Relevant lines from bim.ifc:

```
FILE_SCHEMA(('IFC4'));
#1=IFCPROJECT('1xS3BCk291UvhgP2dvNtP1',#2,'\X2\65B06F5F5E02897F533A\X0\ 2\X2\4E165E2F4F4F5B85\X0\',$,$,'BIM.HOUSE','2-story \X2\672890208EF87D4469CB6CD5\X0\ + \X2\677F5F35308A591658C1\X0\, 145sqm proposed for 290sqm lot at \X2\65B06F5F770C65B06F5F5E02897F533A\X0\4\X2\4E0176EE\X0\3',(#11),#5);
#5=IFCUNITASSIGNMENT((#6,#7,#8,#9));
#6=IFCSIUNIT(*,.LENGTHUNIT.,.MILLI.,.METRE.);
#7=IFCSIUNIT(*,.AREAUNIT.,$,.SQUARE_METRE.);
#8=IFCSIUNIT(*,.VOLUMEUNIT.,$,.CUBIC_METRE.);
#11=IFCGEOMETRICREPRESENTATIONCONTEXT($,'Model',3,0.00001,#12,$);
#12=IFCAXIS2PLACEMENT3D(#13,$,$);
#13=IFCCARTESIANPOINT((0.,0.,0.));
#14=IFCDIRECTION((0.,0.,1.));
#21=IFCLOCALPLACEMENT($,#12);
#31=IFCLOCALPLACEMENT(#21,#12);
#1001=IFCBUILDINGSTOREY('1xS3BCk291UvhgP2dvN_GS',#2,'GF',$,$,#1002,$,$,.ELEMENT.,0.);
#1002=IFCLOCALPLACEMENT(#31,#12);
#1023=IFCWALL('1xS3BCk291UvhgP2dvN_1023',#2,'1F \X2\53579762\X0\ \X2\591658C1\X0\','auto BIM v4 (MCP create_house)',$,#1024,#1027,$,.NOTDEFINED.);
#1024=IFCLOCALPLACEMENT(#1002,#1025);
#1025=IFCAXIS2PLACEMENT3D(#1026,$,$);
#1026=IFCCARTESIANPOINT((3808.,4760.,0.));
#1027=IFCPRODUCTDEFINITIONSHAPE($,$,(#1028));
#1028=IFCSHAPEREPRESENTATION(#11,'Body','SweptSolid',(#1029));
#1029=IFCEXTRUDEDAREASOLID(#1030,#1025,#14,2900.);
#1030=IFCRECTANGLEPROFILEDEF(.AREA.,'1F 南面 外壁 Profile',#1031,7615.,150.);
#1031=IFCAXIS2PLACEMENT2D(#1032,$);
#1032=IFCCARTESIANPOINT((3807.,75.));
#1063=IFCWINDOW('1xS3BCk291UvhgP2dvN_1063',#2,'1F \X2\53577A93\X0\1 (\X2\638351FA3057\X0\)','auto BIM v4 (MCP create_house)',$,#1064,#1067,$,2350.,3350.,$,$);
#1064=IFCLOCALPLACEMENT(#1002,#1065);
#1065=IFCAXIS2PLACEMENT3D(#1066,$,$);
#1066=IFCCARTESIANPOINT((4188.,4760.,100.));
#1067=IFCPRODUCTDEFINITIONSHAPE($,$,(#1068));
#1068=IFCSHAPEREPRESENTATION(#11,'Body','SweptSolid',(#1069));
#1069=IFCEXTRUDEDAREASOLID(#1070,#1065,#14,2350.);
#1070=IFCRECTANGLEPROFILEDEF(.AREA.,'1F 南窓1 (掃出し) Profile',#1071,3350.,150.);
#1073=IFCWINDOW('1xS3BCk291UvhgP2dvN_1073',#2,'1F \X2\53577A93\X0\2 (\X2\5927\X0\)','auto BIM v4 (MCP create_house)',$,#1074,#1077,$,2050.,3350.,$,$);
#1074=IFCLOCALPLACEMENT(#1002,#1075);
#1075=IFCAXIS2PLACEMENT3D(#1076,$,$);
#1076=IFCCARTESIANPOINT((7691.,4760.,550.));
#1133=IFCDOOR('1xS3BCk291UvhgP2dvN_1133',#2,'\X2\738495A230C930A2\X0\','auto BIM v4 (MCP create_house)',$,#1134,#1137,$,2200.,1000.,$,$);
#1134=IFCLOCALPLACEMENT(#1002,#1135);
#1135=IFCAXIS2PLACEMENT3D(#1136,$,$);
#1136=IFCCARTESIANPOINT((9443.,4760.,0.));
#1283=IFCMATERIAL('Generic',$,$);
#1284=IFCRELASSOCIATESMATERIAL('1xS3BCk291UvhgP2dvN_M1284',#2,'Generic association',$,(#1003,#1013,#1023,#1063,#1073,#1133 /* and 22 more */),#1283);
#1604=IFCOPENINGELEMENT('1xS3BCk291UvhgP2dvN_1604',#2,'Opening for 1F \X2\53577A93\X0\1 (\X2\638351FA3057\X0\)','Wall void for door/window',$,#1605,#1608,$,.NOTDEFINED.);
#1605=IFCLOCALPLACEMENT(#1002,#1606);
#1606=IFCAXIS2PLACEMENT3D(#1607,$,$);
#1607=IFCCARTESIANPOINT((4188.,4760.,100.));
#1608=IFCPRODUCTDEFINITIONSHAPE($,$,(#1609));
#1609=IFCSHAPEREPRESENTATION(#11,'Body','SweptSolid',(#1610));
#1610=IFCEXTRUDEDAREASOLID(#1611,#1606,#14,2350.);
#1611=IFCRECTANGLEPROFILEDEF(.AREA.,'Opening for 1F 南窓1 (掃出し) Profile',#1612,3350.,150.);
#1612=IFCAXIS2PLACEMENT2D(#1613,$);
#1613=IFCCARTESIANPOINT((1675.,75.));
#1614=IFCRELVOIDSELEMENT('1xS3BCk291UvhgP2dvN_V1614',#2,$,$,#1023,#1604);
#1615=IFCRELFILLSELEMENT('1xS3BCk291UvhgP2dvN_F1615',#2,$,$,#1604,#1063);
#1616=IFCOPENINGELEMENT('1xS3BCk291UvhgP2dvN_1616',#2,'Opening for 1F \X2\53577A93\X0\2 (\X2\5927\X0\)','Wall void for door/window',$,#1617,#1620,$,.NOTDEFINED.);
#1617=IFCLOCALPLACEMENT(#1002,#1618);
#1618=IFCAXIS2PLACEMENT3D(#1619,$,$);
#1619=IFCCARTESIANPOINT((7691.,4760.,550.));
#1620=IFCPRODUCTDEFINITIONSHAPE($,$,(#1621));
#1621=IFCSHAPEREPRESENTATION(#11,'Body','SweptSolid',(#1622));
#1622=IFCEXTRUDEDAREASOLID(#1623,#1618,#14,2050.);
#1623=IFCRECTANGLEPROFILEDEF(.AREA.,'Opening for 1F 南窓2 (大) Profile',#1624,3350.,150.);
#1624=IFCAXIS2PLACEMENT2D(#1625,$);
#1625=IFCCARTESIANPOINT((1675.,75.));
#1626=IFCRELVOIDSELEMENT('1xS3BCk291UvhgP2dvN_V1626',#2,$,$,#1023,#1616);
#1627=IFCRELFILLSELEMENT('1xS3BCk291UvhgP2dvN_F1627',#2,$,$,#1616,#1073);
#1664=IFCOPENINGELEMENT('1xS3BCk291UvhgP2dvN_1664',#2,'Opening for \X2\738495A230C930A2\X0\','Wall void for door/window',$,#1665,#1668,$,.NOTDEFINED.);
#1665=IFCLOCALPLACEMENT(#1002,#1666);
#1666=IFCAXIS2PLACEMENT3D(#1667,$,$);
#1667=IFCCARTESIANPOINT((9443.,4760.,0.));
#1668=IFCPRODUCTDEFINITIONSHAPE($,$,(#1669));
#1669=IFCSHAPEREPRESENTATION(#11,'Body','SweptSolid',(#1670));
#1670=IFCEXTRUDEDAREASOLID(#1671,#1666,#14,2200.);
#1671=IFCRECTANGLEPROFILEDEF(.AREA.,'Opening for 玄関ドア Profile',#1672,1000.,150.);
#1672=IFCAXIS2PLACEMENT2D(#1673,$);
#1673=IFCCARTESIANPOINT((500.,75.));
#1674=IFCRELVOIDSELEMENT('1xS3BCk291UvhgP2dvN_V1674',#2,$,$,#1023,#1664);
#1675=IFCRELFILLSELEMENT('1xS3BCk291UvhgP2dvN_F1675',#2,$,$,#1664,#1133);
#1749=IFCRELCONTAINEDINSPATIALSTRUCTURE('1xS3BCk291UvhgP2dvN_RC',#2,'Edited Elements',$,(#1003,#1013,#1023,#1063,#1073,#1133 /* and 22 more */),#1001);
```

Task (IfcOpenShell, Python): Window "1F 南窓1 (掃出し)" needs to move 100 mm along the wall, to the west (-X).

```python
import ifcopenshell
import ifcopenshell.api.geometry
import ifcopenshell.util.placement

model = ifcopenshell.open("bim.ifc")

window = model.by_guid("1xS3BCk291UvhgP2dvN_1063")
opening = window.FillsVoids[0].RelatingOpeningElement
wall = opening.VoidsElements[0].RelatingBuildingElement

wall_matrix = ifcopenshell.util.placement.get_local_placement(wall.ObjectPlacement)
shift = wall_matrix[:3, 0] * -100.0
before = ifcopenshell.util.placement.get_local_placement(window.ObjectPlacement)[:3, 3].copy()

# The window is not placed relative to its opening, so move both.
for product in (opening, window):
    matrix = ifcopenshell.util.placement.get_local_placement(product.ObjectPlacement)
    matrix[:3, 3] += shift
    ifcopenshell.api.geometry.edit_object_placement(model, product=product, matrix=matrix, is_si=False)

after = ifcopenshell.util.placement.get_local_placement(window.ObjectPlacement)[:3, 3]
print("window moved by", (after - before).round(3) + 0.0)

model.write("bim_v2.ifc")
```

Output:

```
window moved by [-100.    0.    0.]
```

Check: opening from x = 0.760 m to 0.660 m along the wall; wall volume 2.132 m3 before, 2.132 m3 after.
